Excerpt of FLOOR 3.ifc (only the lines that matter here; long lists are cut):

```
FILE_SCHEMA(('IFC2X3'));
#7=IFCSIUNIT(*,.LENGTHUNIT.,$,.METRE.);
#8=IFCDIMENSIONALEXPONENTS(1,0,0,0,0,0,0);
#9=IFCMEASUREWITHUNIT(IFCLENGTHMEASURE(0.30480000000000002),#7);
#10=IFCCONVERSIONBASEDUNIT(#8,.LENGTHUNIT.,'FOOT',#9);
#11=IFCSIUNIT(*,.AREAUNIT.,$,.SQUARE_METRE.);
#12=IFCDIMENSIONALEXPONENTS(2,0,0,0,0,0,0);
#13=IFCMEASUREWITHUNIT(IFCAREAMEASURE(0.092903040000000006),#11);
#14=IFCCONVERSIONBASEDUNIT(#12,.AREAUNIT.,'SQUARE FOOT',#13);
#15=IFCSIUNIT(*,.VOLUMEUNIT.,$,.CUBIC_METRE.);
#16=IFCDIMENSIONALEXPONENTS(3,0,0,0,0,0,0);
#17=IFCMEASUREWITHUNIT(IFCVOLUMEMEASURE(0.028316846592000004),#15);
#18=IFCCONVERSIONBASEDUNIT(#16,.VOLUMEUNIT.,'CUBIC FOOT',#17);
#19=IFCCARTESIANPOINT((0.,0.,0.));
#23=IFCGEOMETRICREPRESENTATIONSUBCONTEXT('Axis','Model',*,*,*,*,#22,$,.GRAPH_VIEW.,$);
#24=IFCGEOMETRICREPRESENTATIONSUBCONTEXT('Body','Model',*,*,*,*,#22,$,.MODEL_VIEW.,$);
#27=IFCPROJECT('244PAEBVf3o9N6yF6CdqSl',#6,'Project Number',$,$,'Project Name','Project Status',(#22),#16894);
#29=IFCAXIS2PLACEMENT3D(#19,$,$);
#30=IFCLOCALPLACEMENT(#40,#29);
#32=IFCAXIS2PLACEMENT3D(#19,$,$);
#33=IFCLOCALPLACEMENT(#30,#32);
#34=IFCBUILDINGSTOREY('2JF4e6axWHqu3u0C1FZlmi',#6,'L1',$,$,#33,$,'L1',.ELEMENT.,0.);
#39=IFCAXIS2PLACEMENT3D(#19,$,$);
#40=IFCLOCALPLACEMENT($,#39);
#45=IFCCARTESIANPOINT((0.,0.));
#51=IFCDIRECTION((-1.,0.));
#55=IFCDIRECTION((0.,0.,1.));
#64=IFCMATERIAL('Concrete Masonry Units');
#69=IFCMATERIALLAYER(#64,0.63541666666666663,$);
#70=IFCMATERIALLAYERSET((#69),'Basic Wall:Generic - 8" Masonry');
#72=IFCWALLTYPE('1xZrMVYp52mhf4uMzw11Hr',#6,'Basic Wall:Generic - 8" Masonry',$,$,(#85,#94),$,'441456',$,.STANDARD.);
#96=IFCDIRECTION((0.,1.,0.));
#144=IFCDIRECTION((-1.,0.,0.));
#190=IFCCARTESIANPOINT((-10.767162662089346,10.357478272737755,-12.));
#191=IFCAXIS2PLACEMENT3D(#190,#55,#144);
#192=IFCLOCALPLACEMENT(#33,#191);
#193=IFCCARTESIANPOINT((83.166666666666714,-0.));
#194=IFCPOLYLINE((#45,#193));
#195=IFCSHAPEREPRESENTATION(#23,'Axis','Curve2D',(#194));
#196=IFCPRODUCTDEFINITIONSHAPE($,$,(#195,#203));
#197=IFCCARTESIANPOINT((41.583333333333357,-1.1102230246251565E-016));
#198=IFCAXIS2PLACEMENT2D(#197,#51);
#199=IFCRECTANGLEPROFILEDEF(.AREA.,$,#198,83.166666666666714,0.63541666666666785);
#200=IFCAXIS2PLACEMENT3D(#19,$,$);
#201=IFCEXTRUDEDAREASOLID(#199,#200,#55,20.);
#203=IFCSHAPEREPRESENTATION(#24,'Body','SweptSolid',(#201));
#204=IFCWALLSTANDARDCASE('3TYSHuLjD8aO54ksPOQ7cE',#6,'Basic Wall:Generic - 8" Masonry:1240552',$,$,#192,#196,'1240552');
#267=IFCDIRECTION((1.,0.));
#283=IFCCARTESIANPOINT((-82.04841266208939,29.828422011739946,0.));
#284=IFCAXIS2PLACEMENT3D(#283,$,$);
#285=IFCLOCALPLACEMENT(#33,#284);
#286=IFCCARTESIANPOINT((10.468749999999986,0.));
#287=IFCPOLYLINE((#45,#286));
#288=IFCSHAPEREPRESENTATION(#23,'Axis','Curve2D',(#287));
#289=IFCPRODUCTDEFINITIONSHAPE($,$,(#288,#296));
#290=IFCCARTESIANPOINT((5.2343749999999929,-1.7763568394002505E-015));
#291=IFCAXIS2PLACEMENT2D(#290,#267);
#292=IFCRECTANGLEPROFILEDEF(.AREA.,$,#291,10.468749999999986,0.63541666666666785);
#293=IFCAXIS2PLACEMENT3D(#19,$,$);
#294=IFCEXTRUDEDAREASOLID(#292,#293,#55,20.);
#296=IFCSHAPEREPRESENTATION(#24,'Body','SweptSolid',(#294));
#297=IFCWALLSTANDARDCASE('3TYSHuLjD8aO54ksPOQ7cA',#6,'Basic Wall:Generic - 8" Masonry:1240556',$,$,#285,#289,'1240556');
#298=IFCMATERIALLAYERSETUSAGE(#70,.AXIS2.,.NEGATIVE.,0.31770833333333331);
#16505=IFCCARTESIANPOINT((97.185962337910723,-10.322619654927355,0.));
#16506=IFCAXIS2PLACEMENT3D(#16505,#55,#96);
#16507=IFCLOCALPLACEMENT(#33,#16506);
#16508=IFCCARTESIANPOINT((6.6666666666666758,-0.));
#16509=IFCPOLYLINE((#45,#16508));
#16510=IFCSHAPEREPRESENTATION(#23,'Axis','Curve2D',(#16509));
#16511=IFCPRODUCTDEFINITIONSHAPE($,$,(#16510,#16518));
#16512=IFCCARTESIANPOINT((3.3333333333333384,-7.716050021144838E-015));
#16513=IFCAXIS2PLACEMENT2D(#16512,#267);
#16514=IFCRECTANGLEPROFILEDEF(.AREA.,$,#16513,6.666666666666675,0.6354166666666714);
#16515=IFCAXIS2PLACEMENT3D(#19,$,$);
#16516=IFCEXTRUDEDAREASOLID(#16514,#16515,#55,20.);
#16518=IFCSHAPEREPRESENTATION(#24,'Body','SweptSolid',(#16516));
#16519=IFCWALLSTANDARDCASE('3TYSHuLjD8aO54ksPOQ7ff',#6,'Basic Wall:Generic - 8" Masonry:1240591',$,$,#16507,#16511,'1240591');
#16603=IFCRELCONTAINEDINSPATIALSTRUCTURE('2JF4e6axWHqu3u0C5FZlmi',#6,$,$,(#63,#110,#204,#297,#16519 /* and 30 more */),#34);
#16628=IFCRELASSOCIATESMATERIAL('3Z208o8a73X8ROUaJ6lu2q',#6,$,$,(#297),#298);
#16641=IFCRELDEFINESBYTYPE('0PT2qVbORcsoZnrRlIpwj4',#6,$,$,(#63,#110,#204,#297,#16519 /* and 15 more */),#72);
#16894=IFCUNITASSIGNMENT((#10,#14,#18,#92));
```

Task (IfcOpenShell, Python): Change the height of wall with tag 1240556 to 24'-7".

```python
import ifcopenshell
import ifcopenshell.geom
import ifcopenshell.util.representation
import ifcopenshell.util.shape
import ifcopenshell.util.unit

model = ifcopenshell.open("FLOOR 3.ifc")
unit_scale = ifcopenshell.util.unit.calculate_unit_scale(model)
settings = ifcopenshell.geom.settings()


def volume(element):
    """Net volume in cubic metres, openings subtracted."""
    shape = ifcopenshell.geom.create_shape(settings, element)
    return ifcopenshell.util.shape.get_volume(shape.geometry)


wall = model.by_id(297)
before = volume(wall)

body = ifcopenshell.util.representation.get_representation(wall, "Model", "Body")
solid = body.Items[0]
old_height = solid.Depth
solid.Depth = 295 * 0.0254 / unit_scale
after = volume(wall)

print(f"height {old_height:g} -> {solid.Depth:g}, volume {before:.3f} -> {after:.3f} m3")

model.write("FLOOR 3_rev.ifc")
```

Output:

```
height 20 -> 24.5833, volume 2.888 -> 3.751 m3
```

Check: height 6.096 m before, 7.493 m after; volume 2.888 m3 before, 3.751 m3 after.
